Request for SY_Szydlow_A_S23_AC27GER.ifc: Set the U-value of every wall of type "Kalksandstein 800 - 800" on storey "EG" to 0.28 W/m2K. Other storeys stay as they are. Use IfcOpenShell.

First a look at what the model holds.

```python
import ifcopenshell
import ifcopenshell.util.element

model = ifcopenshell.open("SY_Szydlow_A_S23_AC27GER.ifc")
print(model.schema)
storey = next(s for s in model.by_type("IfcBuildingStorey") if s.Name == "EG")
walls = [e for e in ifcopenshell.util.element.get_decomposition(storey) if e.is_a("IfcWall")]
seen = {}
for e in walls:
    element_type = ifcopenshell.util.element.get_type(e)
    key = (element_type.Name if element_type != e and element_type else None, ifcopenshell.util.element.get_pset(e, "Pset_WallCommon", "ThermalTransmittance"))
    seen[key] = seen.get(key, 0) + 1
for (name, value), count in sorted(seen.items(), key=str):
    print(count, "x", name, "|", value)
```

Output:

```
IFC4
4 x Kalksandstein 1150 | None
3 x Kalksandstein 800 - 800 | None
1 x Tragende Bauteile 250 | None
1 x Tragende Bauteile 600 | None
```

```python
import ifcopenshell
import ifcopenshell.api.pset
import ifcopenshell.util.element

model = ifcopenshell.open("SY_Szydlow_A_S23_AC27GER.ifc")

storey = next(s for s in model.by_type("IfcBuildingStorey") if s.Name == "EG")
walls = [e for e in ifcopenshell.util.element.get_decomposition(storey) if e.is_a("IfcWall")]

count = 0
for e in walls:
    element_type = ifcopenshell.util.element.get_type(e)
    if element_type in (None, e) or element_type.Name != "Kalksandstein 800 - 800":
        continue
    # add_pset returns the element's existing set when there is one.
    pset = ifcopenshell.api.pset.add_pset(model, product=e, name="Pset_WallCommon")
    ifcopenshell.api.pset.edit_pset(model, pset=pset, properties={"ThermalTransmittance": 0.28})
    count += 1

print(count, "walls updated")

model.write("SY_Szydlow_A_S23_AC27GER_rev.ifc")
```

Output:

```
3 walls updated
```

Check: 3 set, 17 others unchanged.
